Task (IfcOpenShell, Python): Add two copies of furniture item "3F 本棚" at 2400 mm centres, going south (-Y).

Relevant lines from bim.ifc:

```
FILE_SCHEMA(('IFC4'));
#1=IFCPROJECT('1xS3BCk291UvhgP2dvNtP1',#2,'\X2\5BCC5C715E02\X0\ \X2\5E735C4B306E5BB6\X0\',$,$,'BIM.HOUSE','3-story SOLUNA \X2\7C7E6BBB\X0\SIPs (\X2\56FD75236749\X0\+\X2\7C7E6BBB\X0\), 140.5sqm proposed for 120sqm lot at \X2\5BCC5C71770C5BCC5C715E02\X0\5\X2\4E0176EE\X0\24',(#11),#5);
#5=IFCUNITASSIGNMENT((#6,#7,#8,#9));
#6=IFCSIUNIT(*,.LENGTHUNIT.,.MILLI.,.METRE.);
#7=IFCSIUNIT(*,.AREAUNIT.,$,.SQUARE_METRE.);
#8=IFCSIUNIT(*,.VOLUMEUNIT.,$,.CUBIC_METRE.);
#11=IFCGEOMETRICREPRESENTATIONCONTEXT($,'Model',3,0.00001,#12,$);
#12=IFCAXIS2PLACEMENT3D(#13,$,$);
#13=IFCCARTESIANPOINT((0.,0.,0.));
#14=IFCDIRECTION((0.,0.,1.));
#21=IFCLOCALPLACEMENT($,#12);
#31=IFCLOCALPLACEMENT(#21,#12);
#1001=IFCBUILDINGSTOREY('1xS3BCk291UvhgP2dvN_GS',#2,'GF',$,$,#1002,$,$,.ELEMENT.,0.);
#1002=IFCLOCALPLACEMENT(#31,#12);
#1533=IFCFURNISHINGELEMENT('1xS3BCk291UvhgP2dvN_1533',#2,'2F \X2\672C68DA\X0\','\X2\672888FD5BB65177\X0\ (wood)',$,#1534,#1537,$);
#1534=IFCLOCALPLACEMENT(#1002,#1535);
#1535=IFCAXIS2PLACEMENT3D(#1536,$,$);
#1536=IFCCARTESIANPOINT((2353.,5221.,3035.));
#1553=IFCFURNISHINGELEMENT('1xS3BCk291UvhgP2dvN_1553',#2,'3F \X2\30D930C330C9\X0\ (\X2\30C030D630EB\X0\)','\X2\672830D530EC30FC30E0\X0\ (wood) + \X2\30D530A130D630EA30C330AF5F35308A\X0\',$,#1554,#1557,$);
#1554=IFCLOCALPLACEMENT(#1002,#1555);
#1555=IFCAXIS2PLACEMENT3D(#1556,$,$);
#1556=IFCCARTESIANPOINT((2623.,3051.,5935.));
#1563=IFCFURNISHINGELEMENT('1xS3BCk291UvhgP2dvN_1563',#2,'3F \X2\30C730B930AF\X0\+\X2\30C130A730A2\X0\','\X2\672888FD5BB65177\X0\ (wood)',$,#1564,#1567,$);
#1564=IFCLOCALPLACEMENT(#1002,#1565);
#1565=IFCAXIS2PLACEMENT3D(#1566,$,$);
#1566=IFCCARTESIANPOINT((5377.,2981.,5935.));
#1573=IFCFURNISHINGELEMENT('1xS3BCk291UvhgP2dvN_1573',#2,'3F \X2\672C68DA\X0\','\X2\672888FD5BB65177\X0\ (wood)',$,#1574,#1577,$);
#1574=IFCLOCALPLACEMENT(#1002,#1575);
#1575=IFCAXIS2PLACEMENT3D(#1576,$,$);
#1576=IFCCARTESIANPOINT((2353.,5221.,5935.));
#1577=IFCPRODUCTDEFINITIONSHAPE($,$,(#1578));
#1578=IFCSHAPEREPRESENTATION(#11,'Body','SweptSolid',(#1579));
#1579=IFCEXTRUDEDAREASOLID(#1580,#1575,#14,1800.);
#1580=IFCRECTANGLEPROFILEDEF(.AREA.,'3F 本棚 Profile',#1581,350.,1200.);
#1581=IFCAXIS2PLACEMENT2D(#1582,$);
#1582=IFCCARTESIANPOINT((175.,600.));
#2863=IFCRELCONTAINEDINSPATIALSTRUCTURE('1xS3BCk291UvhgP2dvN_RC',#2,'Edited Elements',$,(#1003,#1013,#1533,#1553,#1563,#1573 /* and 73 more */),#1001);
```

```python
import numpy as np
import ifcopenshell
import ifcopenshell.api.geometry
import ifcopenshell.api.root
import ifcopenshell.util.element
import ifcopenshell.util.placement
import ifcopenshell.util.unit

model = ifcopenshell.open("bim.ifc")
unit_scale = ifcopenshell.util.unit.calculate_unit_scale(model)


def reuse_history(source, copy):
    """copy_class also copies each property set's owner history, people and application; keep the originals."""
    for rel in copy.IsDefinedBy:
        if rel.is_a("IfcRelDefinesByProperties") and (history := rel.RelatingPropertyDefinition.OwnerHistory):
            rel.RelatingPropertyDefinition.OwnerHistory = source.OwnerHistory
            ifcopenshell.util.element.remove_deep2(model, history)


source = model.by_id(1573)
base = ifcopenshell.util.placement.get_local_placement(source.ObjectPlacement)
step = np.array([0.0, -1.0, 0.0]) * 2.4 / unit_scale

for i in range(1, 3):
    copy = ifcopenshell.api.root.copy_class(model, product=source)
    copy.Representation = ifcopenshell.util.element.copy_deep(
        model, source.Representation, exclude=["IfcGeometricRepresentationContext", "IfcRepresentationMap"]
    )
    reuse_history(source, copy)
    matrix = base.copy()
    matrix[:3, 3] += i * step
    print("added at", matrix[:3, 3].round(3) + 0.0)
    ifcopenshell.api.geometry.edit_object_placement(model, product=copy, matrix=matrix, is_si=False)

model.write("bim-out.ifc")
```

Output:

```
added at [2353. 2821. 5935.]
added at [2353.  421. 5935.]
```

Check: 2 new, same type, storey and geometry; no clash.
